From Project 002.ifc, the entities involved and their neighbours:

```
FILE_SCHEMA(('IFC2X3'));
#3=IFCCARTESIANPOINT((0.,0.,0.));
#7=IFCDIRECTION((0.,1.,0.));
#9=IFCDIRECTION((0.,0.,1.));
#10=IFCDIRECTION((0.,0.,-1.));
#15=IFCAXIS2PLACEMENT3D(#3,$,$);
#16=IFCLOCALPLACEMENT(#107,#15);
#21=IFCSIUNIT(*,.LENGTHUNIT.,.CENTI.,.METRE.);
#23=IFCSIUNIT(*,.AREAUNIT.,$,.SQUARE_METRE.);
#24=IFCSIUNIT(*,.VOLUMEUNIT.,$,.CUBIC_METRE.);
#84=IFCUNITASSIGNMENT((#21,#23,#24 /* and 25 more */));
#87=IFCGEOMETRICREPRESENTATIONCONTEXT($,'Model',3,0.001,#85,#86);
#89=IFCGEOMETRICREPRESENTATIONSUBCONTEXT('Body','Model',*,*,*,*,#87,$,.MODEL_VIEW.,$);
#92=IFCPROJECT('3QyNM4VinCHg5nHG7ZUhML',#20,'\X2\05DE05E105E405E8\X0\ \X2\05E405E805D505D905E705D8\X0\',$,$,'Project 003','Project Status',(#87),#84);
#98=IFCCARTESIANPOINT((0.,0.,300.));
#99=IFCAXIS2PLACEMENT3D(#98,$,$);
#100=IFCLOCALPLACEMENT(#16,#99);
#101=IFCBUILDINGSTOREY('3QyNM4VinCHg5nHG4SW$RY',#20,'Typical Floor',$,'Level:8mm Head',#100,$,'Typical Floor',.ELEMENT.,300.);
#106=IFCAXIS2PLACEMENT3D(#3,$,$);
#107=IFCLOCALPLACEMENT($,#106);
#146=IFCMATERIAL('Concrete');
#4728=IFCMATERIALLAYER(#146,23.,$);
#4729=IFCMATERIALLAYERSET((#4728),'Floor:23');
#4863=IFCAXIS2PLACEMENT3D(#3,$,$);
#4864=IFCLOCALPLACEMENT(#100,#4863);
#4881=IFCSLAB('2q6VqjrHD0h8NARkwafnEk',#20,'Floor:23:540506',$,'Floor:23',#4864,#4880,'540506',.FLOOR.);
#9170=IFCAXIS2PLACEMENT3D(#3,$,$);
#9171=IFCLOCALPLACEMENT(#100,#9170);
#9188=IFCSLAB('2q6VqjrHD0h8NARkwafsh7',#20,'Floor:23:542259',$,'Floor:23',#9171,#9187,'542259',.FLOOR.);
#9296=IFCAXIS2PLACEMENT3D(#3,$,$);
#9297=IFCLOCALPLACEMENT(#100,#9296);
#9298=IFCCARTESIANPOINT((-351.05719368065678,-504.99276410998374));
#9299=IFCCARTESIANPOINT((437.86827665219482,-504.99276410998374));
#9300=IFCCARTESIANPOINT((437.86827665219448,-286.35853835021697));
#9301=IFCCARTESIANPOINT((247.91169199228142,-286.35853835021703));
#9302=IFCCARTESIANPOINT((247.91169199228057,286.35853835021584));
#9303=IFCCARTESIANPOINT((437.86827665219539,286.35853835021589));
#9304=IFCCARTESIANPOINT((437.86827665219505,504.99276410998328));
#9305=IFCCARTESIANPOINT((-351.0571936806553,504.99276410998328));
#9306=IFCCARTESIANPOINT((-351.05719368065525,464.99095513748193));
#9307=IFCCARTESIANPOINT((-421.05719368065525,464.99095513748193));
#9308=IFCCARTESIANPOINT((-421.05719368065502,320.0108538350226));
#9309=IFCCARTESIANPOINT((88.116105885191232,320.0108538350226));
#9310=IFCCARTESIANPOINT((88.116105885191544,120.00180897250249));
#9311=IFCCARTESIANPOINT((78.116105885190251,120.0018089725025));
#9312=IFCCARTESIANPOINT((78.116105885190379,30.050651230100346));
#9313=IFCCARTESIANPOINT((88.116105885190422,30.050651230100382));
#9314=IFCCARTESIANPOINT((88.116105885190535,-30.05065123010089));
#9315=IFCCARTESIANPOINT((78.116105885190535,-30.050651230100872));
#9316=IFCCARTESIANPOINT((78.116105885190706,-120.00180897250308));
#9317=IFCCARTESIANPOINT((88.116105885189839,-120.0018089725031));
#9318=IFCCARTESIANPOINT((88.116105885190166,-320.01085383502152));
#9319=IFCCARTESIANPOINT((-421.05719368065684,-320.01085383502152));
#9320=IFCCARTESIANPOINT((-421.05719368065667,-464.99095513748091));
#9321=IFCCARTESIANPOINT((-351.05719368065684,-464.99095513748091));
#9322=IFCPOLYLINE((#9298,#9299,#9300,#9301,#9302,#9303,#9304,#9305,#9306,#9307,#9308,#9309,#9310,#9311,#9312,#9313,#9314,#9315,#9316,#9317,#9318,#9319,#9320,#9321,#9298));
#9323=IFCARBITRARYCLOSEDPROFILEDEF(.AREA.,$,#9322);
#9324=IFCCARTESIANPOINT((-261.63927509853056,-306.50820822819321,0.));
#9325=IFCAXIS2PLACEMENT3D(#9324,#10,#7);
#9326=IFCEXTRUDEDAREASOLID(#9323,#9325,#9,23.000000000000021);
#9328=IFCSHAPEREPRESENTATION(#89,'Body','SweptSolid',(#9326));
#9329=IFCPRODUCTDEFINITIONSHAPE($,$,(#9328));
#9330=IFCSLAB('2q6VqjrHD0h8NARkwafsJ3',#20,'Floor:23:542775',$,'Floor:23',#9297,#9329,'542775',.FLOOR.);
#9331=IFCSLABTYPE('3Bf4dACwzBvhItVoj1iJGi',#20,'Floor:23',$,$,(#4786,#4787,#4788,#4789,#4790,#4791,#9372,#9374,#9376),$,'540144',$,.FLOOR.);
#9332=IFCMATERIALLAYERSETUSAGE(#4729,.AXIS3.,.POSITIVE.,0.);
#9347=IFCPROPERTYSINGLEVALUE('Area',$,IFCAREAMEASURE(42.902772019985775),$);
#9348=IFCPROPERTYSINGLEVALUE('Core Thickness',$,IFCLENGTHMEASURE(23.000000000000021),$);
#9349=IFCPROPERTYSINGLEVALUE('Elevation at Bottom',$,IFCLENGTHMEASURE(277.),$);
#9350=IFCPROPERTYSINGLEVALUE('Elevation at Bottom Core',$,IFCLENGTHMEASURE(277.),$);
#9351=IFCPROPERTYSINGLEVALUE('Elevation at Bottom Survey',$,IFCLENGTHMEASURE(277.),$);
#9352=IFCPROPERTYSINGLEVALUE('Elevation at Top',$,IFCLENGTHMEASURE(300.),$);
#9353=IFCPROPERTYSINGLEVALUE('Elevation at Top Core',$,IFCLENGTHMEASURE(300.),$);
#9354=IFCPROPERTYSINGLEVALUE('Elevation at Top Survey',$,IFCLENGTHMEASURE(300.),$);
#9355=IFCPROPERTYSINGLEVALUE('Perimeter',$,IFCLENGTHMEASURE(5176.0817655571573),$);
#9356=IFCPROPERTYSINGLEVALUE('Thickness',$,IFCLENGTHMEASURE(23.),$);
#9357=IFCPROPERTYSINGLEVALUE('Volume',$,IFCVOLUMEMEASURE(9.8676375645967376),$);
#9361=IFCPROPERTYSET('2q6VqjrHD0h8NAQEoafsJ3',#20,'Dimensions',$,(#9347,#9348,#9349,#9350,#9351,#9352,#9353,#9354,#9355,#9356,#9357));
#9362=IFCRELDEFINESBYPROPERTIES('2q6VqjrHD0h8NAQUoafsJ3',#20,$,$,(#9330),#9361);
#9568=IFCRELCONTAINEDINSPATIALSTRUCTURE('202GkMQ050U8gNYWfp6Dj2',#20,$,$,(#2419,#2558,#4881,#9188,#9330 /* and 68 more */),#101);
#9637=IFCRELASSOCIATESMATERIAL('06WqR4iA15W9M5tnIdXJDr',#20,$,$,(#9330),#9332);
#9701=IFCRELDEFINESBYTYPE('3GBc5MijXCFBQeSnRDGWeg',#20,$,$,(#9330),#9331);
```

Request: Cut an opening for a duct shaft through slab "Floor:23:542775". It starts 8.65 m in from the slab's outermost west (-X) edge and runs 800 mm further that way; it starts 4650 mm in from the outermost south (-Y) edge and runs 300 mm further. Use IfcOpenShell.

```python
import numpy as np
import ifcopenshell
import ifcopenshell.api.feature
import ifcopenshell.api.geometry
import ifcopenshell.api.pset
import ifcopenshell.api.root
import ifcopenshell.geom
import ifcopenshell.util.element
import ifcopenshell.util.placement
import ifcopenshell.util.representation
import ifcopenshell.util.shape
import ifcopenshell.util.unit

model = ifcopenshell.open("Project 002.ifc")
unit_scale = ifcopenshell.util.unit.calculate_unit_scale(model)
area_scale = ifcopenshell.util.unit.calculate_unit_scale(model, "AREAUNIT")
volume_scale = ifcopenshell.util.unit.calculate_unit_scale(model, "VOLUMEUNIT")
settings = ifcopenshell.geom.settings()


def volume(element):
    """Net volume in cubic metres, openings subtracted."""
    shape = ifcopenshell.geom.create_shape(settings, element)
    return ifcopenshell.util.shape.get_volume(shape.geometry)


slab = model.by_guid("2q6VqjrHD0h8NARkwafsJ3")
before = volume(slab)

# Extent in the slab's own axes, in metres. The edges named are its -X and -Y sides.
slab_shape = ifcopenshell.geom.create_shape(settings, slab)
vertices = ifcopenshell.util.shape.get_vertices(slab_shape.geometry)
x_min, y_min, bottom = vertices.min(axis=0)
top = vertices[:, 2].max()

opening = ifcopenshell.api.root.create_entity(model, ifc_class="IfcOpeningElement", name="Duct shaft opening")
context = ifcopenshell.util.representation.get_context(model, "Model", "Body", "MODEL_VIEW")
width, depth = 0.8, 0.3
outline = [(0.0, 0.0), (width, 0.0), (width, depth), (0.0, depth), (0.0, 0.0)]
# Overshoot both faces by 50 mm so the cut is clean.
shape = ifcopenshell.api.geometry.add_slab_representation(
    model, context=context, depth=top - bottom + 0.1, polyline=outline
)
ifcopenshell.api.geometry.assign_representation(model, product=opening, representation=shape)

matrix = ifcopenshell.util.placement.get_local_placement(slab.ObjectPlacement)
matrix[:, 3] = matrix @ np.append(np.array([x_min + 8.65, y_min + 4.65, bottom - 0.05]) / unit_scale, 1.0)
ifcopenshell.api.geometry.edit_object_placement(model, product=opening, matrix=matrix, is_si=False)
ifcopenshell.api.feature.add_feature(model, feature=opening, element=slab)

after = volume(slab)

# Update the slab's stored quantities.
pset = model.by_id(ifcopenshell.util.element.get_pset(slab, "Dimensions", should_inherit=False)["id"])
ifcopenshell.api.pset.edit_pset(model, pset=pset, properties={
    "Area": model.create_entity("IfcAreaMeasure", after / (top - bottom) / area_scale),
    "Volume": model.create_entity("IfcVolumeMeasure", after / volume_scale),
})

print(f"slab volume {before:.3f} -> {after:.3f} m3")

model.write("Project 002-out.ifc")
```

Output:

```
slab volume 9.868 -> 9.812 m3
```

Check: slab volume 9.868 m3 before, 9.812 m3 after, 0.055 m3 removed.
